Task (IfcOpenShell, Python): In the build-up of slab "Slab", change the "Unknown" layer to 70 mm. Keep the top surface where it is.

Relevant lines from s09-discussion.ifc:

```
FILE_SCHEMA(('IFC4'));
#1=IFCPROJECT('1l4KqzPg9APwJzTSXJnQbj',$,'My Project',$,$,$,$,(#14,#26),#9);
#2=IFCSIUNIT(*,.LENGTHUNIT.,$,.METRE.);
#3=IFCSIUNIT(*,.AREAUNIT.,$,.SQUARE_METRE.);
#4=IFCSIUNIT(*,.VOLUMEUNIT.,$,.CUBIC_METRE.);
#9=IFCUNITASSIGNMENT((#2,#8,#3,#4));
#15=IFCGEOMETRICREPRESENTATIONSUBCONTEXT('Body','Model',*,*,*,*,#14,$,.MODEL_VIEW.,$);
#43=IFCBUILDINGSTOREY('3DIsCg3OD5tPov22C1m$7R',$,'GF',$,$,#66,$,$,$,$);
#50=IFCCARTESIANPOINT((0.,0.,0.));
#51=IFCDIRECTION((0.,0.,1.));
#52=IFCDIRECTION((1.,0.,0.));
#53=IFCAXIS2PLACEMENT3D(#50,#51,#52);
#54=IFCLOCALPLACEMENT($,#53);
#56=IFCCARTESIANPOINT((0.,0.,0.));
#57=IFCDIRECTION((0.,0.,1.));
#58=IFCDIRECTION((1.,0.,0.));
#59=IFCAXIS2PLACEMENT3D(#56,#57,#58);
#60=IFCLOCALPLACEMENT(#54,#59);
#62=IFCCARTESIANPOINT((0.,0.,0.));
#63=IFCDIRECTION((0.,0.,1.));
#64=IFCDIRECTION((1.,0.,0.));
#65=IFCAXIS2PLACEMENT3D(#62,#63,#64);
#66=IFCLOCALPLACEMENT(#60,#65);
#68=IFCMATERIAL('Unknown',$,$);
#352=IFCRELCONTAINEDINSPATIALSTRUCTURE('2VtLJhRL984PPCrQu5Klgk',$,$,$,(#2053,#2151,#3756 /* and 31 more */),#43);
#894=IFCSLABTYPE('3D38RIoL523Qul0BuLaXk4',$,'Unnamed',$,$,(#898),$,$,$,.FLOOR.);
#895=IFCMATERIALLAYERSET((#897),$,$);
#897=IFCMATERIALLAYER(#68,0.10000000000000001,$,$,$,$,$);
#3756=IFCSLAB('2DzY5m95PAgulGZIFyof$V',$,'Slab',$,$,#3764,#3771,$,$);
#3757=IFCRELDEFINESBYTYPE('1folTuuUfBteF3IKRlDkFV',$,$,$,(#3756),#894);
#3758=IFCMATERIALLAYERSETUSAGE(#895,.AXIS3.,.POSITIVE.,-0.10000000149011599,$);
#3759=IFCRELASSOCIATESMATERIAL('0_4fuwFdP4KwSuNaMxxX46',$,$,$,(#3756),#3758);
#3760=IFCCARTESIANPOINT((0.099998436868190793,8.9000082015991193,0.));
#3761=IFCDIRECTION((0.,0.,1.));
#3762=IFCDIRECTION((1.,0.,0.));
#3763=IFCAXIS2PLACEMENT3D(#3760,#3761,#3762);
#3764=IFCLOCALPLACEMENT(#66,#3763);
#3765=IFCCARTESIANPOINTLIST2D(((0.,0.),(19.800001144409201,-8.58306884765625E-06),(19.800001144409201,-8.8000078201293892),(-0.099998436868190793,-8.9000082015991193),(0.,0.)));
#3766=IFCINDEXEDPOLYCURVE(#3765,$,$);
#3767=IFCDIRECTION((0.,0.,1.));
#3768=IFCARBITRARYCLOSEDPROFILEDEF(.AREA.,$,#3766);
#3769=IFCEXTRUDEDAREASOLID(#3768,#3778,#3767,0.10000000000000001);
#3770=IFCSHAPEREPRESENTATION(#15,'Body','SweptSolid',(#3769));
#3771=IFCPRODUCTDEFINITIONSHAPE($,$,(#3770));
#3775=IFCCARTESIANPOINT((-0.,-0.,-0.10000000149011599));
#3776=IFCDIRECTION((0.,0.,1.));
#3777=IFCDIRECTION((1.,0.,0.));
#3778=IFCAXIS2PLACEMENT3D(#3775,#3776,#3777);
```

```python
import ifcopenshell
import ifcopenshell.util.element
import ifcopenshell.util.representation

model = ifcopenshell.open("s09-discussion.ifc")

layer_set = model.by_id(895)
layer = next(l for l in layer_set.MaterialLayers if l.Material and l.Material.Name == "Unknown")
change = 0.07 - layer.LayerThickness
layer.LayerThickness += change

# Geometry does not follow the layer set by itself.
slabs = [e for e in ifcopenshell.util.element.get_elements_by_material(model, layer_set) if e.is_a("IfcSlab")]
for slab in sorted(slabs, key=lambda e: e.id()):
    body = ifcopenshell.util.representation.get_representation(slab, "Model", "Body")
    solid = body.Items[0]
    old_depth = solid.Depth
    solid.Depth += change
    # Extruded upwards: lower the start of the extrusion so the top stays.
    x, y, z = solid.Position.Location.Coordinates
    solid.Position.Location = model.createIfcCartesianPoint((x, y, z - change))
    print(slab.id(), f"{old_depth:g} -> {solid.Depth:g}")

# The layers are counted up from the underside, which has moved.
for usage in {ifcopenshell.util.element.get_material(slab) for slab in slabs}:
    usage.OffsetFromReferenceLine -= change

model.write("s09-discussion_updated.ifc")
```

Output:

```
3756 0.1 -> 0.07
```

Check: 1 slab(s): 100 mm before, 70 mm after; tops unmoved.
